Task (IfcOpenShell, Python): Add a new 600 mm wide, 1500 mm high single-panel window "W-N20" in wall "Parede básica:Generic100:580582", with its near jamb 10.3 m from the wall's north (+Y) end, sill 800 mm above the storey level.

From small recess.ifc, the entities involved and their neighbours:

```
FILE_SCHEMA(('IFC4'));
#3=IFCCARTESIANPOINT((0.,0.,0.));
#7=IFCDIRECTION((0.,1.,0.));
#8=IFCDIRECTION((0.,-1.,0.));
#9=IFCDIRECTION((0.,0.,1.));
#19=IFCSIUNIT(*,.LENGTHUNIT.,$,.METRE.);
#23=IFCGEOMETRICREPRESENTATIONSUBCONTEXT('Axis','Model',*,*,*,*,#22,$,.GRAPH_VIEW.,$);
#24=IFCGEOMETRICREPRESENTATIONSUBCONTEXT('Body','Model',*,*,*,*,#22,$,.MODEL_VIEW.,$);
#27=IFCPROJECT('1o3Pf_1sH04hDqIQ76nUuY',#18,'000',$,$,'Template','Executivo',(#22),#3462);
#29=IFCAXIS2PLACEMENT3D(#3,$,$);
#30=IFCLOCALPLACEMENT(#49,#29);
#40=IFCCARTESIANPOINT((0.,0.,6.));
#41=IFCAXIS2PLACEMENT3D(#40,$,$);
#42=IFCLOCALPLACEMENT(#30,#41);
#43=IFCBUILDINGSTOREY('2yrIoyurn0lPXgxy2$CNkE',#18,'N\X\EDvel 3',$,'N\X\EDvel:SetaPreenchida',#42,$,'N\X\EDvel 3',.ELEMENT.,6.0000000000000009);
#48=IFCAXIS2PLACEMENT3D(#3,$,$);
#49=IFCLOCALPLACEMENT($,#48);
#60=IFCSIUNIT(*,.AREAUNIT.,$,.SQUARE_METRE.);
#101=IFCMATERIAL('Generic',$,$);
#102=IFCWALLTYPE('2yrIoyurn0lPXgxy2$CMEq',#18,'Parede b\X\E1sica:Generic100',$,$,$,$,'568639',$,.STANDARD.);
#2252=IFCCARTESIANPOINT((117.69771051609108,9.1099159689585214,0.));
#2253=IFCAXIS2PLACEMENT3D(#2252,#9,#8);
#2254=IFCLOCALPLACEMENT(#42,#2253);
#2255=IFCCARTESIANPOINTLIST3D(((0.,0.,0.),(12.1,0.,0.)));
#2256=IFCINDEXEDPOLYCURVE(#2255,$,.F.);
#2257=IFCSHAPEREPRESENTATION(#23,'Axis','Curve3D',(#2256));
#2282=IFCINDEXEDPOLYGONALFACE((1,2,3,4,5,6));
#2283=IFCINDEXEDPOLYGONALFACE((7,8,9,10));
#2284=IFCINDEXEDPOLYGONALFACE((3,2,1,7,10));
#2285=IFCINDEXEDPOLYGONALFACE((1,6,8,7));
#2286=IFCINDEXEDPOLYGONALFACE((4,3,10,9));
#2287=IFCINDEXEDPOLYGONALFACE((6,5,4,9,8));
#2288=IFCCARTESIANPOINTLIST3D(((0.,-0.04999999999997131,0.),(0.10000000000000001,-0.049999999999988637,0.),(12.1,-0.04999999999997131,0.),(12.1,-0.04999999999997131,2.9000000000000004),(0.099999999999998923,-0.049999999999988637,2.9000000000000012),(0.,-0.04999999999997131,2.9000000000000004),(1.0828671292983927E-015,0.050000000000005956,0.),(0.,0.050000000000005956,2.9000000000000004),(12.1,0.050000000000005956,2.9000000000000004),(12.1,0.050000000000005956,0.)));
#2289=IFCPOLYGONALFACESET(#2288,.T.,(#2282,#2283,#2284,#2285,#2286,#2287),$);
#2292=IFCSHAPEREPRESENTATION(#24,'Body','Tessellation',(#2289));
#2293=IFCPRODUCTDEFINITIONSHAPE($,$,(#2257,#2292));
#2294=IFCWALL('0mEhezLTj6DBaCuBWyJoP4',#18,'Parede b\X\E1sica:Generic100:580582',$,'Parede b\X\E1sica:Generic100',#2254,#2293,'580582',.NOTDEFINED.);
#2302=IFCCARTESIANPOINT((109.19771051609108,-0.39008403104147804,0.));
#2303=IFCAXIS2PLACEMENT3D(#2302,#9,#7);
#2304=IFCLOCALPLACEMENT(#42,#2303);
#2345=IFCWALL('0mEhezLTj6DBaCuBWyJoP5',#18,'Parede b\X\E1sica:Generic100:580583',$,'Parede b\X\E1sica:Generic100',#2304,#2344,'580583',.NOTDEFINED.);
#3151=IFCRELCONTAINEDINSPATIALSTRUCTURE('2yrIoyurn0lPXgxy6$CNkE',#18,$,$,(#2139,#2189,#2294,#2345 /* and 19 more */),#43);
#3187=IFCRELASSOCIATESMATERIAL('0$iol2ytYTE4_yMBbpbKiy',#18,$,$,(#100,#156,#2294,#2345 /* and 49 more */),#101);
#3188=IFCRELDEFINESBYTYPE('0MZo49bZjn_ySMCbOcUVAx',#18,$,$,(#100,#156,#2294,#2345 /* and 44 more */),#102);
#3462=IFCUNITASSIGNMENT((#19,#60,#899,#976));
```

```python
import numpy as np
import ifcopenshell
import ifcopenshell.api.feature
import ifcopenshell.api.geometry
import ifcopenshell.api.root
import ifcopenshell.api.spatial
import ifcopenshell.geom
import ifcopenshell.util.element
import ifcopenshell.util.placement
import ifcopenshell.util.representation
import ifcopenshell.util.shape
import ifcopenshell.util.unit

model = ifcopenshell.open("small recess.ifc")
unit_scale = ifcopenshell.util.unit.calculate_unit_scale(model)
settings = ifcopenshell.geom.settings()


def volume(element):
    """Net volume in cubic metres, openings subtracted."""
    shape = ifcopenshell.geom.create_shape(settings, element)
    return ifcopenshell.util.shape.get_volume(shape.geometry)


wall = model.by_id(2294)
storey = ifcopenshell.util.element.get_container(wall, ifc_class="IfcBuildingStorey")
context = ifcopenshell.util.representation.get_context(model, "Model", "Body", "MODEL_VIEW")
before = volume(wall)

width, height, from_end, sill = 0.6, 1.5, 10.3, 0.8  # metres

# The wall runs along its own X axis, and the end named is its -X end.
wall_shape = ifcopenshell.geom.create_shape(settings, wall)
x, y, z = ifcopenshell.util.shape.get_vertices(wall_shape.geometry).T
start = x.min() + from_end
face, thickness = float(y.min()), float(y.max() - y.min())
wall_matrix = ifcopenshell.util.placement.get_local_placement(wall.ObjectPlacement)
level = ifcopenshell.util.placement.get_local_placement(storey.ObjectPlacement)[2, 3]


def in_wall(x, y):
    """Placement at x, y metres in the wall's axes, at sill height."""
    matrix = wall_matrix.copy()
    matrix[:, 3] = wall_matrix @ np.array([x / unit_scale, y / unit_scale, 0.0, 1.0])
    matrix[2, 3] = level + sill / unit_scale
    return matrix


# Opening: a box that overshoots both wall faces by 50 mm.
opening = ifcopenshell.api.root.create_entity(model, ifc_class="IfcOpeningElement", predefined_type="OPENING")
box = ifcopenshell.api.geometry.add_wall_representation(
    model, context=context, length=width, height=height, thickness=thickness + 0.1
)
ifcopenshell.api.geometry.assign_representation(model, product=opening, representation=box)
ifcopenshell.api.geometry.edit_object_placement(model, product=opening, matrix=in_wall(start, face - 0.05), is_si=False)
ifcopenshell.api.feature.add_feature(model, feature=opening, element=wall)

window = ifcopenshell.api.root.create_entity(model, ifc_class="IfcWindow", name="W-N20", predefined_type="WINDOW")
window.OverallWidth, window.OverallHeight = width / unit_scale, height / unit_scale
window.PartitioningType = "SINGLE_PANEL"
body = ifcopenshell.api.geometry.add_window_representation(
    model,
    context=context,
    overall_width=window.OverallWidth,
    overall_height=window.OverallHeight,
    partition_type="SINGLE_PANEL",
)
ifcopenshell.api.geometry.assign_representation(model, product=window, representation=body)
ifcopenshell.api.spatial.assign_container(model, products=[window], relating_structure=storey)
ifcopenshell.api.feature.add_filling(model, opening=opening, element=window)

# Centre the window in the wall's thickness.
ifcopenshell.api.geometry.edit_object_placement(model, product=window, matrix=in_wall(start, face), is_si=False)
window_shape = ifcopenshell.geom.create_shape(settings, window)
depth = ifcopenshell.util.shape.get_vertices(window_shape.geometry)[:, 1]
offset = face + thickness / 2 - (depth.min() + depth.max()) / 2
ifcopenshell.api.geometry.edit_object_placement(model, product=window, matrix=in_wall(start, offset), is_si=False)

after = volume(wall)

print(f"wall volume {before:.3f} -> {after:.3f} m3")

model.write("small recess_edited.ifc")
```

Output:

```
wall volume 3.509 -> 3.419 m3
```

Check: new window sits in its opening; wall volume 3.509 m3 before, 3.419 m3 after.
